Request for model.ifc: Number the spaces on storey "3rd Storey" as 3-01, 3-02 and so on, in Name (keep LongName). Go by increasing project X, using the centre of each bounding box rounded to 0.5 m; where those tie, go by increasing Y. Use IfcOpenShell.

First a look at what the model holds.

```python
import ifcopenshell
import ifcopenshell.util.element
import ifcopenshell.util.placement

model = ifcopenshell.open("model.ifc")
print(model.schema)
storey = next(s for s in model.by_type("IfcBuildingStorey") if s.Name == "3rd Storey")
spaces = [e for e in ifcopenshell.util.element.get_decomposition(storey) if e.is_a("IfcSpace")]
for e in sorted(spaces, key=lambda e: e.id()):
    origin = ifcopenshell.util.placement.get_local_placement(e.ObjectPlacement)[:3, 3]
    print(e.id(), e.Name, e.LongName, origin.round(2) + 0.0, sep=" | ")
```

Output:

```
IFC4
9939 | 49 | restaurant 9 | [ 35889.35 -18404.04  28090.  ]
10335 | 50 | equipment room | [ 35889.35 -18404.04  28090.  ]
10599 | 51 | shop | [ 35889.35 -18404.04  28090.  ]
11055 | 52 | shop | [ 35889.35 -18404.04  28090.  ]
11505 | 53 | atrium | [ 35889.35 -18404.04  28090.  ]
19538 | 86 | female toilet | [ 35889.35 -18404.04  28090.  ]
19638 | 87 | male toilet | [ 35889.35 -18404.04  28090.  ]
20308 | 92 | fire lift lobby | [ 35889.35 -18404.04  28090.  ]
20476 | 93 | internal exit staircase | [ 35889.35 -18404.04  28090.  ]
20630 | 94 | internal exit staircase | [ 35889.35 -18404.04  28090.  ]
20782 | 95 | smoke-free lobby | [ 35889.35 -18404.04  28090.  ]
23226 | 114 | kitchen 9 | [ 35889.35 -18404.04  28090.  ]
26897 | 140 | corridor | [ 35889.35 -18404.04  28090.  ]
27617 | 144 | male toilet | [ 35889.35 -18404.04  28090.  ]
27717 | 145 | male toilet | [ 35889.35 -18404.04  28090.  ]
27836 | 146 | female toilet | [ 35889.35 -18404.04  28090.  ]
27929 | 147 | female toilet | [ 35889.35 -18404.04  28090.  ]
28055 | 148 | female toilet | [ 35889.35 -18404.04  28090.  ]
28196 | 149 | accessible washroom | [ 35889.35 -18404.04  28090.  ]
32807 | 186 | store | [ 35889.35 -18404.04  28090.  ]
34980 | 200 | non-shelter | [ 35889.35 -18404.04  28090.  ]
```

```python
import ifcopenshell
import ifcopenshell.geom
import ifcopenshell.util.element
import ifcopenshell.util.shape

model = ifcopenshell.open("model.ifc")
settings = ifcopenshell.geom.settings()
settings.set("use-world-coords", True)


def centre(element):
    shape = ifcopenshell.geom.create_shape(settings, element)
    return ifcopenshell.util.shape.get_bbox_centroid(shape.geometry)


storey = next(s for s in model.by_type("IfcBuildingStorey") if s.Name == "3rd Storey")
spaces = [e for e in ifcopenshell.util.element.get_decomposition(storey) if e.is_a("IfcSpace")]

# Insertion points can sit at a corner or the storey origin, so sort by the geometry (in metres).
centres = {e: centre(e) for e in spaces}
spaces.sort(key=lambda e: (round(centres[e][0] / 0.5), centres[e][1]))

for i, e in enumerate(spaces, start=1):
    number = f"3-{i:02d}"
    e.Name = number
    print(e.id(), number)

model.write("model_v2.ifc")
```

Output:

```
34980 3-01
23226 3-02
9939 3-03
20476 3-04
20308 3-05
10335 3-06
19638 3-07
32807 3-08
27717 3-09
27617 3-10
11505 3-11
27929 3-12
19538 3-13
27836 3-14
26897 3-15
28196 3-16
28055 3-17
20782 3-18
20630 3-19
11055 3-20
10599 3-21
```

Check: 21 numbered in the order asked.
